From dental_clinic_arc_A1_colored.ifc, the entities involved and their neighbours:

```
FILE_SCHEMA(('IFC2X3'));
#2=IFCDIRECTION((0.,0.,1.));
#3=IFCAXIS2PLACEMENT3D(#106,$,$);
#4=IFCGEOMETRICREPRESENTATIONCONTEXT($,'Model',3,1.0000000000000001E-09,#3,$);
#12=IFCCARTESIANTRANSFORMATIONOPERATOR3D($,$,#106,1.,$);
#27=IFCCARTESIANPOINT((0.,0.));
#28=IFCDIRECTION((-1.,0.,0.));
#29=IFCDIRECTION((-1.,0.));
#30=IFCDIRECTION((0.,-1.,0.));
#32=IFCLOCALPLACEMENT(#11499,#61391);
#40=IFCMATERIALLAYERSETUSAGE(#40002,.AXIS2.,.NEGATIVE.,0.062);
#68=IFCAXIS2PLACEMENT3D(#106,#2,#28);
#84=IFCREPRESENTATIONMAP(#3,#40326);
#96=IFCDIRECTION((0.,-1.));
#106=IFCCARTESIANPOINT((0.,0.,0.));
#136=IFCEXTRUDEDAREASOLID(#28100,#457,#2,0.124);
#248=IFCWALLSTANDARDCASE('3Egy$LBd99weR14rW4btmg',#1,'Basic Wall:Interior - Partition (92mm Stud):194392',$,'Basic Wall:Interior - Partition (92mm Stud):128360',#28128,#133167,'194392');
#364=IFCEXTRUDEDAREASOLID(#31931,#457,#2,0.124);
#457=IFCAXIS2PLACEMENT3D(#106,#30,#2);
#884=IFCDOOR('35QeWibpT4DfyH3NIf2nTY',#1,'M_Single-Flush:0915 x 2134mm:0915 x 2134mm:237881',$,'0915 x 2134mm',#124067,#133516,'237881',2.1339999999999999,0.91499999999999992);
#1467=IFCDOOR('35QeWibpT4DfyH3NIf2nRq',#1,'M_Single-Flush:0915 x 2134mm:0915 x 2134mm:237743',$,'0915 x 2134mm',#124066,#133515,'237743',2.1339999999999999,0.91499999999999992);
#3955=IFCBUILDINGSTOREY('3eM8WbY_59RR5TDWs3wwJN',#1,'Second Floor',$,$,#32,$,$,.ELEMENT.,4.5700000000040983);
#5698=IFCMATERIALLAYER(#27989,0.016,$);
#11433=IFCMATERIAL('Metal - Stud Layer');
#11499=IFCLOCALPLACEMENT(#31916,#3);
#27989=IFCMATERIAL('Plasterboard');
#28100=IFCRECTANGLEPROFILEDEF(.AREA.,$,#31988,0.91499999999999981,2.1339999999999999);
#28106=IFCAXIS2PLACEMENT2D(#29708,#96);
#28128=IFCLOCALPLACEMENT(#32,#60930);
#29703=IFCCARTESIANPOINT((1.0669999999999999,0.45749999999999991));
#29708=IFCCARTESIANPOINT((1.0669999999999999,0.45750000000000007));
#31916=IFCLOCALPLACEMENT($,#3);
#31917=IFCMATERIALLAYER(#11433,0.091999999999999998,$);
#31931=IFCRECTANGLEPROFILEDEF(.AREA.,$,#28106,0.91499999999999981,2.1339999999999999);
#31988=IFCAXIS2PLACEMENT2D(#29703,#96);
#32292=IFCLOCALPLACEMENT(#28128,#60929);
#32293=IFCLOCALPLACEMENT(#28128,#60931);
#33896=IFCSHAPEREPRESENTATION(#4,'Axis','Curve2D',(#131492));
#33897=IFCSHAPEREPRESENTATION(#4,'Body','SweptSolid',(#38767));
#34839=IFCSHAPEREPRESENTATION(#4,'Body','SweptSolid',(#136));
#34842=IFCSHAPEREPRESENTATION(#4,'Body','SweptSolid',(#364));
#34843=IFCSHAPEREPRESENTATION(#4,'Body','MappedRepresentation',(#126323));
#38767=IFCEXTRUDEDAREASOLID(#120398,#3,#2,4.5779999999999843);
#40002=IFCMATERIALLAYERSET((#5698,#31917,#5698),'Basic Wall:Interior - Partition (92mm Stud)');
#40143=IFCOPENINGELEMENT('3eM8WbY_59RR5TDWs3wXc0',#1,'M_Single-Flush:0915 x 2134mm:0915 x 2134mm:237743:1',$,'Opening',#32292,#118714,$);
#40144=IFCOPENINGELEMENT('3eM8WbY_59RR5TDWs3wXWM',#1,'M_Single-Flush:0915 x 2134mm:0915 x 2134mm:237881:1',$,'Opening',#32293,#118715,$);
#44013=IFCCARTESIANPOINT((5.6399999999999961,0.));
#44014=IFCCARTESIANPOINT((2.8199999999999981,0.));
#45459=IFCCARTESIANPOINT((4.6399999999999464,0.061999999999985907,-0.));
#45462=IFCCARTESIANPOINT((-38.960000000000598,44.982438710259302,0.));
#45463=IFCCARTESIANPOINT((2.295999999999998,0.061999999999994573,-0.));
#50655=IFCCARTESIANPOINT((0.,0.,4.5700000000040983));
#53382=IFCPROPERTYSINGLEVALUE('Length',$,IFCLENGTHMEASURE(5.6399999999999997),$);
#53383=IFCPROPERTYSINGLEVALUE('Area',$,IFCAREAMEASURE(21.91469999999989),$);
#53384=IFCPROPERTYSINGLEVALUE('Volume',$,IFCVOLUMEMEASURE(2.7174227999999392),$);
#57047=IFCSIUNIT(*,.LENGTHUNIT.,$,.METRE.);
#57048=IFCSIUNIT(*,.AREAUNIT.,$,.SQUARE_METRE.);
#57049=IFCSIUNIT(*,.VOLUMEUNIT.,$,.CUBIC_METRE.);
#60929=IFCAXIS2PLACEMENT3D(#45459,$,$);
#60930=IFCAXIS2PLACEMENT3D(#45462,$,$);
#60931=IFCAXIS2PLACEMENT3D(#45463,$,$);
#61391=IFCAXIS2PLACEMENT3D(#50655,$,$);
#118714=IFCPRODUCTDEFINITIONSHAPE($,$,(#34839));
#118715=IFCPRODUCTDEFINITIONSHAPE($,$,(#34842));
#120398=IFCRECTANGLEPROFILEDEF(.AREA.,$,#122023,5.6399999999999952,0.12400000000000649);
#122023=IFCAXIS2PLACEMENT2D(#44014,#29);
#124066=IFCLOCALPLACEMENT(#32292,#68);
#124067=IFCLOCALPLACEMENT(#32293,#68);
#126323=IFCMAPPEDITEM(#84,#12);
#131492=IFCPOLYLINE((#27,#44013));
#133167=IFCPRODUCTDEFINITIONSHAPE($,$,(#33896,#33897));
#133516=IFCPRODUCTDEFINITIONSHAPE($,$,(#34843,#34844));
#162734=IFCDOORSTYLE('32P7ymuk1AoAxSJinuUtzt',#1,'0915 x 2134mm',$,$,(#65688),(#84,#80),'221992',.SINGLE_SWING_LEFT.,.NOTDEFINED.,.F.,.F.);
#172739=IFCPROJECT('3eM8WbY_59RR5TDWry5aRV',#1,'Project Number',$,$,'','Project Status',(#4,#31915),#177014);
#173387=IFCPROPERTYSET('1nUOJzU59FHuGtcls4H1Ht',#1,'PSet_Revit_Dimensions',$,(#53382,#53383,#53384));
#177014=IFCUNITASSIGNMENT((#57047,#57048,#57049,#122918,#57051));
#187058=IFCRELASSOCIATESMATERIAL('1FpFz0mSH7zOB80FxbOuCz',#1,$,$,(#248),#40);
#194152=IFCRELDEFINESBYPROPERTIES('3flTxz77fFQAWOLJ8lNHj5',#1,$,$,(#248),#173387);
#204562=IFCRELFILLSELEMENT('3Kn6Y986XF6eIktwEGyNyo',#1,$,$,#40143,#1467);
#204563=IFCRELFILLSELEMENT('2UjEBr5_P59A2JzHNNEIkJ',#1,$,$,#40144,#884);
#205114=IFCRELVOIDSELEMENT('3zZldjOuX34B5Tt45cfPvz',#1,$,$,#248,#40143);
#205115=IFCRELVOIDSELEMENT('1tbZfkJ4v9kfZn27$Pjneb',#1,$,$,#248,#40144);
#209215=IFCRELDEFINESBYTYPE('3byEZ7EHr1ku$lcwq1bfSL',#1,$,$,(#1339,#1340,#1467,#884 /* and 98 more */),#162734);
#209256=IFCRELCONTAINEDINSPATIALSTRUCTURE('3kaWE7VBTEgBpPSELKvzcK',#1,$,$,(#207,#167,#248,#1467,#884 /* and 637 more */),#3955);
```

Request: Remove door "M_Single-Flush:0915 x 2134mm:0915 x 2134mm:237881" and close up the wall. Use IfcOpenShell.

```python
import ifcopenshell
import ifcopenshell.api.feature
import ifcopenshell.api.pset
import ifcopenshell.api.root
import ifcopenshell.geom
import ifcopenshell.util.element
import ifcopenshell.util.shape
import ifcopenshell.util.unit

model = ifcopenshell.open("dental_clinic_arc_A1_colored.ifc")
area_scale = ifcopenshell.util.unit.calculate_unit_scale(model, "AREAUNIT")
volume_scale = ifcopenshell.util.unit.calculate_unit_scale(model, "VOLUMEUNIT")
settings = ifcopenshell.geom.settings()


def volume(element):
    """Net volume in cubic metres, openings subtracted."""
    shape = ifcopenshell.geom.create_shape(settings, element)
    return ifcopenshell.util.shape.get_volume(shape.geometry)


door = model.by_guid("35QeWibpT4DfyH3NIf2nTY")
opening = door.FillsVoids[0].RelatingOpeningElement
wall = opening.VoidsElements[0].RelatingBuildingElement
before = volume(wall)

ifcopenshell.api.root.remove_product(model, product=door)
ifcopenshell.api.feature.remove_feature(model, feature=opening)

after = volume(wall)
thickness = 0.124  # wall thickness in metres

# Update the wall's stored quantities.
pset = model.by_id(ifcopenshell.util.element.get_pset(wall, "PSet_Revit_Dimensions", should_inherit=False)["id"])
ifcopenshell.api.pset.edit_pset(model, pset=pset, properties={
    "Area": model.create_entity("IfcAreaMeasure", after / thickness / area_scale),
    "Volume": model.create_entity("IfcVolumeMeasure", after / volume_scale),
})

print(f"wall volume {before:.3f} -> {after:.3f} m3")

model.write("dental_clinic_arc_A1_colored_rev.ifc")
```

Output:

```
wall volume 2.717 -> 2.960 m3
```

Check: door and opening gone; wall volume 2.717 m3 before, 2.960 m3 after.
